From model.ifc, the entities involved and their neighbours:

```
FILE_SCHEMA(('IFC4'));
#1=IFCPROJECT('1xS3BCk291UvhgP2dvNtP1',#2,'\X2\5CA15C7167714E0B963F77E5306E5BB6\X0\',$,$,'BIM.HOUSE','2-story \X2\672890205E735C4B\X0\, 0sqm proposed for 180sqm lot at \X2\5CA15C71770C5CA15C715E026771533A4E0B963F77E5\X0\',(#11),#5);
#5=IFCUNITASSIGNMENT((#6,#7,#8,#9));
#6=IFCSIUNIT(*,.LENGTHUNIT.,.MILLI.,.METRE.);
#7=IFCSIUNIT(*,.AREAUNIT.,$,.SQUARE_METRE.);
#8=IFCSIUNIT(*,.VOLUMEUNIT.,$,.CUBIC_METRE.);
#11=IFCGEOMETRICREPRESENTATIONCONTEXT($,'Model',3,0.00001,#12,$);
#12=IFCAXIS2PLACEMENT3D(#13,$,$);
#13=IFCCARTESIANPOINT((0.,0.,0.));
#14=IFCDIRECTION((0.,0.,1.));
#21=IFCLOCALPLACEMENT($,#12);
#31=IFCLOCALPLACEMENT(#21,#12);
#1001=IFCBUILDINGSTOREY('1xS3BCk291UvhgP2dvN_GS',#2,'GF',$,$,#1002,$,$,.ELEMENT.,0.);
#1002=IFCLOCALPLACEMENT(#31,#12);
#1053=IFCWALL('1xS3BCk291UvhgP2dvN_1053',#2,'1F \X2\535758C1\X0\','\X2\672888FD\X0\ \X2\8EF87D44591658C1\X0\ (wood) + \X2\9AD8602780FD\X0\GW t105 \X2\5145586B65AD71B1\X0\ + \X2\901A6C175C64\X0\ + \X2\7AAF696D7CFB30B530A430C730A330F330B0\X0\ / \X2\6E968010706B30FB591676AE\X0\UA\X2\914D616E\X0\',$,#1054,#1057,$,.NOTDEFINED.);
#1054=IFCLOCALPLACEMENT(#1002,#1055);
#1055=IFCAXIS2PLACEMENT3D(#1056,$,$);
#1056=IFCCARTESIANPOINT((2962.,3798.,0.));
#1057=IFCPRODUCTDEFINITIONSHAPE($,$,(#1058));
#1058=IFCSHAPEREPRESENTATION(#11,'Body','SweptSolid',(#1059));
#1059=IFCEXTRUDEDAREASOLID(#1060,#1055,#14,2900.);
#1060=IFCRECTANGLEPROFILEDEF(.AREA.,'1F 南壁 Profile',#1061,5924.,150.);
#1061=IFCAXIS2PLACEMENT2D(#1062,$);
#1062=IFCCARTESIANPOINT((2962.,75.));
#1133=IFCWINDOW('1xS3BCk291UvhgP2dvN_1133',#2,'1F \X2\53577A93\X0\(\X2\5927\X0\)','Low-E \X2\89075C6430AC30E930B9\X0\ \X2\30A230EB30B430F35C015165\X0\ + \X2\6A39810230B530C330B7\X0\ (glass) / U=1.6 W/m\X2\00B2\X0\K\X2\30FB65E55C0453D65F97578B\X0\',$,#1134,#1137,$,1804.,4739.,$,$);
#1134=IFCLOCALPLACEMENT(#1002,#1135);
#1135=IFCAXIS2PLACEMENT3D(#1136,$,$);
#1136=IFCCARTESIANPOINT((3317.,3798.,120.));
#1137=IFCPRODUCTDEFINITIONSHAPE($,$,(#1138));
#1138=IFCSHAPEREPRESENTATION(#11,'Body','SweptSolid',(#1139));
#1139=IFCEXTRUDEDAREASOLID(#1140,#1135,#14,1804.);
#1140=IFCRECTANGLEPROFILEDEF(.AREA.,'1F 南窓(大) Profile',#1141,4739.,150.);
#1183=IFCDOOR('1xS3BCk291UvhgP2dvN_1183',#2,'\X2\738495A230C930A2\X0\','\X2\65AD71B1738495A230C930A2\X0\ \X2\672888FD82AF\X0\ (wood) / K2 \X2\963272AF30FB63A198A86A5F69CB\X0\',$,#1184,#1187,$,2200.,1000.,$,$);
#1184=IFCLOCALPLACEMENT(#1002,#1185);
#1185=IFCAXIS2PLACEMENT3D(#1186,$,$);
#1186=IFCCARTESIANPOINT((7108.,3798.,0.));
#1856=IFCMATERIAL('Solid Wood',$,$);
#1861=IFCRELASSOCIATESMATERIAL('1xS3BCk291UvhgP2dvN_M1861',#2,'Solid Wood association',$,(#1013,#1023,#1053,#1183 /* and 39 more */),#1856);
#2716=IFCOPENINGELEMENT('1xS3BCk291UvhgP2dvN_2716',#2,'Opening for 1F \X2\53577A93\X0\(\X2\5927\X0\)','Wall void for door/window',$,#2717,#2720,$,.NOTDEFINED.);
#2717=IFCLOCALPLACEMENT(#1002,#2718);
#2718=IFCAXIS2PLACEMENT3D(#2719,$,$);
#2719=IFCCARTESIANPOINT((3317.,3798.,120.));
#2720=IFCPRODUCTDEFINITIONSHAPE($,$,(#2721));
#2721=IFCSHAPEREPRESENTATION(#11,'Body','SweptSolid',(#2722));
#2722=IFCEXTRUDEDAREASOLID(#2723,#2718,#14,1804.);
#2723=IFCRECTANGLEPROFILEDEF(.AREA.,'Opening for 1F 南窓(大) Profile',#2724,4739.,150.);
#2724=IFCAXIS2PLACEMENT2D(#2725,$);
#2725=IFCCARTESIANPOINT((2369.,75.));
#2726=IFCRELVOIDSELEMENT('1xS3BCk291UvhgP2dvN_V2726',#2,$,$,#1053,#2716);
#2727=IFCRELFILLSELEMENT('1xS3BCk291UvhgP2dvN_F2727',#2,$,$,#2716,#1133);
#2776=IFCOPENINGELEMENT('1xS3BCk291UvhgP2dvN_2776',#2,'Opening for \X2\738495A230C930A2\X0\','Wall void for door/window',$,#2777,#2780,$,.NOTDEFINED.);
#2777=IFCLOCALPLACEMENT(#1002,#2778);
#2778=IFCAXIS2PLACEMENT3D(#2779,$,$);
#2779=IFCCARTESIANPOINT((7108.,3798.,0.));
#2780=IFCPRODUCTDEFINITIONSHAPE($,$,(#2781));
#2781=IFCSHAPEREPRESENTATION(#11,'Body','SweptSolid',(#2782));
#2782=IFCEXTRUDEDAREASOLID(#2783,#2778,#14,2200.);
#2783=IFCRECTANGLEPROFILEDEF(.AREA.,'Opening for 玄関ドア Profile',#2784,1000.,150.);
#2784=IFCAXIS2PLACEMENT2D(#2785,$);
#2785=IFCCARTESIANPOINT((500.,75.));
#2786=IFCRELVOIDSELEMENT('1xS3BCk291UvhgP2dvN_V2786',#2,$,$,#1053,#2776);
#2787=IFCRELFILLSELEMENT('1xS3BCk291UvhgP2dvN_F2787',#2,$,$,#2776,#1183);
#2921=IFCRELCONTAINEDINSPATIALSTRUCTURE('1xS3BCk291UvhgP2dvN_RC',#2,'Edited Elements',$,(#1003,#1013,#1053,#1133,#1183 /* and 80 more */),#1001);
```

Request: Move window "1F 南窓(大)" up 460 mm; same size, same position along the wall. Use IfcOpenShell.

```python
import numpy as np
import ifcopenshell
import ifcopenshell.api.geometry
import ifcopenshell.util.placement
import ifcopenshell.util.unit

model = ifcopenshell.open("model.ifc")
unit_scale = ifcopenshell.util.unit.calculate_unit_scale(model)

window = model.by_guid("1xS3BCk291UvhgP2dvN_1133")
opening = window.FillsVoids[0].RelatingOpeningElement
dz = 0.46 / unit_scale

shift = np.array([0.0, 0.0, dz])
# The window is not placed relative to its opening, so move both.
for product in (opening, window):
    matrix = ifcopenshell.util.placement.get_local_placement(product.ObjectPlacement)
    matrix[:3, 3] += shift
    ifcopenshell.api.geometry.edit_object_placement(model, product=product, matrix=matrix, is_si=False)

print(f"moved by {dz * unit_scale:+.3f} m")

model.write("model_updated.ifc")
```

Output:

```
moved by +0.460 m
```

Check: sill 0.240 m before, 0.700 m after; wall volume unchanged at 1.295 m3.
